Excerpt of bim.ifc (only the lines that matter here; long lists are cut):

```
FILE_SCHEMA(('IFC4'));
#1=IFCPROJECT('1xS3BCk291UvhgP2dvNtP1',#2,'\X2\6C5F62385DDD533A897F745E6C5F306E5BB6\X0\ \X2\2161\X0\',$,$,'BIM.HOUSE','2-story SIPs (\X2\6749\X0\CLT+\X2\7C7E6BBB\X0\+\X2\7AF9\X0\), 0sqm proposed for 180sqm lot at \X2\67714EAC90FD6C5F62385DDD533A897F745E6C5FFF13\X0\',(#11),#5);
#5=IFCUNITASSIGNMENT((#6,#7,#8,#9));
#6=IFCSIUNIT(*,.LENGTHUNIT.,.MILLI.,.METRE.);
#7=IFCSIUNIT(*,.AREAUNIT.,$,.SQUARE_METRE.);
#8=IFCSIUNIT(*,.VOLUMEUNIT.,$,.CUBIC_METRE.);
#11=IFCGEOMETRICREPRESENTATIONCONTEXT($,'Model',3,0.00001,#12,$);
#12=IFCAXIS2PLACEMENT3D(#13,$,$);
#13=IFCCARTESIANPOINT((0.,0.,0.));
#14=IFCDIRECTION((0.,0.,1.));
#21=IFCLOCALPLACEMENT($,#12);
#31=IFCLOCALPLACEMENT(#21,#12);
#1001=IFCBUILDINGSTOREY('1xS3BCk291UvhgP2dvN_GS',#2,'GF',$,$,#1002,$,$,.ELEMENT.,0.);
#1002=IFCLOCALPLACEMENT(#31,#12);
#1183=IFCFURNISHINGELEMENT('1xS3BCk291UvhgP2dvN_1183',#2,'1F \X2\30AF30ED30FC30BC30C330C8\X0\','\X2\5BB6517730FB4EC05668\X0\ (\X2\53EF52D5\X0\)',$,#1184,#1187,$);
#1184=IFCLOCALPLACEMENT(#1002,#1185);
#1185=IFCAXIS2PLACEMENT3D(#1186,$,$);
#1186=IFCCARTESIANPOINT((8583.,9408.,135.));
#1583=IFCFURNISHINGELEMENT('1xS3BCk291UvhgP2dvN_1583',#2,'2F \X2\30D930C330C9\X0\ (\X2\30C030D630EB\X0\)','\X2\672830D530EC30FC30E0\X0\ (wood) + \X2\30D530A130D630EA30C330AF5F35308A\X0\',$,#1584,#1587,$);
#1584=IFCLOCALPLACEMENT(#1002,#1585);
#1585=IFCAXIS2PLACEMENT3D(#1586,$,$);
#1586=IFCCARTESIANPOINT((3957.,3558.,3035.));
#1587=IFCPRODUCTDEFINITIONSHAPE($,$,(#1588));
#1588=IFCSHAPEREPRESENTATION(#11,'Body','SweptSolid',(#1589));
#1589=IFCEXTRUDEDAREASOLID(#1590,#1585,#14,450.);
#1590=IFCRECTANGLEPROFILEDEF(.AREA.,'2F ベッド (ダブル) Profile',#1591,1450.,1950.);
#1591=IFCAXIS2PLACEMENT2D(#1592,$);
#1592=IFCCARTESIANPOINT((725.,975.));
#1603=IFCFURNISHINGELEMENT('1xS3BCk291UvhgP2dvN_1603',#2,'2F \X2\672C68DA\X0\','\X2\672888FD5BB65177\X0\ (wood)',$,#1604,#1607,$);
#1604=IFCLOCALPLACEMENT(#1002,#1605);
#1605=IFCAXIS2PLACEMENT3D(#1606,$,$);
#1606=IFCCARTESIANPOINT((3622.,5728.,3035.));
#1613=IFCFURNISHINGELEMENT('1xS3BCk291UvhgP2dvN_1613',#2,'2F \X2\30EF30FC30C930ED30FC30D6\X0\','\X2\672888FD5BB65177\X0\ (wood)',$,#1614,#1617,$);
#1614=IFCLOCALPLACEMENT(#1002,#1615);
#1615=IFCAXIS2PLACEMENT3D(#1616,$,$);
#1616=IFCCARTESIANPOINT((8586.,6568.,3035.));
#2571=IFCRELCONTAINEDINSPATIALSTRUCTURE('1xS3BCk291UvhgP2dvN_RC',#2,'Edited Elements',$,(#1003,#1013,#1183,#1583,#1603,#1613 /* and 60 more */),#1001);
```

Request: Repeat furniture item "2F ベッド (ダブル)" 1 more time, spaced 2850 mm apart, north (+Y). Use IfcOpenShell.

```python
import numpy as np
import ifcopenshell
import ifcopenshell.api.geometry
import ifcopenshell.api.root
import ifcopenshell.util.element
import ifcopenshell.util.placement
import ifcopenshell.util.unit

model = ifcopenshell.open("bim.ifc")
unit_scale = ifcopenshell.util.unit.calculate_unit_scale(model)


def reuse_history(source, copy):
    """copy_class also copies each property set's owner history, people and application; keep the originals."""
    for rel in copy.IsDefinedBy:
        if rel.is_a("IfcRelDefinesByProperties") and (history := rel.RelatingPropertyDefinition.OwnerHistory):
            rel.RelatingPropertyDefinition.OwnerHistory = source.OwnerHistory
            ifcopenshell.util.element.remove_deep2(model, history)


source = model.by_guid("1xS3BCk291UvhgP2dvN_1583")
base = ifcopenshell.util.placement.get_local_placement(source.ObjectPlacement)
step = np.array([0.0, 1.0, 0.0]) * 2.85 / unit_scale

for i in range(1, 2):
    copy = ifcopenshell.api.root.copy_class(model, product=source)
    copy.Representation = ifcopenshell.util.element.copy_deep(
        model, source.Representation, exclude=["IfcGeometricRepresentationContext", "IfcRepresentationMap"]
    )
    reuse_history(source, copy)
    matrix = base.copy()
    matrix[:3, 3] += i * step
    print("added at", matrix[:3, 3].round(3) + 0.0)
    ifcopenshell.api.geometry.edit_object_placement(model, product=copy, matrix=matrix, is_si=False)

model.write("bim_updated.ifc")
```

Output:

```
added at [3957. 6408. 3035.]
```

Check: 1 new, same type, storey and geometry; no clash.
